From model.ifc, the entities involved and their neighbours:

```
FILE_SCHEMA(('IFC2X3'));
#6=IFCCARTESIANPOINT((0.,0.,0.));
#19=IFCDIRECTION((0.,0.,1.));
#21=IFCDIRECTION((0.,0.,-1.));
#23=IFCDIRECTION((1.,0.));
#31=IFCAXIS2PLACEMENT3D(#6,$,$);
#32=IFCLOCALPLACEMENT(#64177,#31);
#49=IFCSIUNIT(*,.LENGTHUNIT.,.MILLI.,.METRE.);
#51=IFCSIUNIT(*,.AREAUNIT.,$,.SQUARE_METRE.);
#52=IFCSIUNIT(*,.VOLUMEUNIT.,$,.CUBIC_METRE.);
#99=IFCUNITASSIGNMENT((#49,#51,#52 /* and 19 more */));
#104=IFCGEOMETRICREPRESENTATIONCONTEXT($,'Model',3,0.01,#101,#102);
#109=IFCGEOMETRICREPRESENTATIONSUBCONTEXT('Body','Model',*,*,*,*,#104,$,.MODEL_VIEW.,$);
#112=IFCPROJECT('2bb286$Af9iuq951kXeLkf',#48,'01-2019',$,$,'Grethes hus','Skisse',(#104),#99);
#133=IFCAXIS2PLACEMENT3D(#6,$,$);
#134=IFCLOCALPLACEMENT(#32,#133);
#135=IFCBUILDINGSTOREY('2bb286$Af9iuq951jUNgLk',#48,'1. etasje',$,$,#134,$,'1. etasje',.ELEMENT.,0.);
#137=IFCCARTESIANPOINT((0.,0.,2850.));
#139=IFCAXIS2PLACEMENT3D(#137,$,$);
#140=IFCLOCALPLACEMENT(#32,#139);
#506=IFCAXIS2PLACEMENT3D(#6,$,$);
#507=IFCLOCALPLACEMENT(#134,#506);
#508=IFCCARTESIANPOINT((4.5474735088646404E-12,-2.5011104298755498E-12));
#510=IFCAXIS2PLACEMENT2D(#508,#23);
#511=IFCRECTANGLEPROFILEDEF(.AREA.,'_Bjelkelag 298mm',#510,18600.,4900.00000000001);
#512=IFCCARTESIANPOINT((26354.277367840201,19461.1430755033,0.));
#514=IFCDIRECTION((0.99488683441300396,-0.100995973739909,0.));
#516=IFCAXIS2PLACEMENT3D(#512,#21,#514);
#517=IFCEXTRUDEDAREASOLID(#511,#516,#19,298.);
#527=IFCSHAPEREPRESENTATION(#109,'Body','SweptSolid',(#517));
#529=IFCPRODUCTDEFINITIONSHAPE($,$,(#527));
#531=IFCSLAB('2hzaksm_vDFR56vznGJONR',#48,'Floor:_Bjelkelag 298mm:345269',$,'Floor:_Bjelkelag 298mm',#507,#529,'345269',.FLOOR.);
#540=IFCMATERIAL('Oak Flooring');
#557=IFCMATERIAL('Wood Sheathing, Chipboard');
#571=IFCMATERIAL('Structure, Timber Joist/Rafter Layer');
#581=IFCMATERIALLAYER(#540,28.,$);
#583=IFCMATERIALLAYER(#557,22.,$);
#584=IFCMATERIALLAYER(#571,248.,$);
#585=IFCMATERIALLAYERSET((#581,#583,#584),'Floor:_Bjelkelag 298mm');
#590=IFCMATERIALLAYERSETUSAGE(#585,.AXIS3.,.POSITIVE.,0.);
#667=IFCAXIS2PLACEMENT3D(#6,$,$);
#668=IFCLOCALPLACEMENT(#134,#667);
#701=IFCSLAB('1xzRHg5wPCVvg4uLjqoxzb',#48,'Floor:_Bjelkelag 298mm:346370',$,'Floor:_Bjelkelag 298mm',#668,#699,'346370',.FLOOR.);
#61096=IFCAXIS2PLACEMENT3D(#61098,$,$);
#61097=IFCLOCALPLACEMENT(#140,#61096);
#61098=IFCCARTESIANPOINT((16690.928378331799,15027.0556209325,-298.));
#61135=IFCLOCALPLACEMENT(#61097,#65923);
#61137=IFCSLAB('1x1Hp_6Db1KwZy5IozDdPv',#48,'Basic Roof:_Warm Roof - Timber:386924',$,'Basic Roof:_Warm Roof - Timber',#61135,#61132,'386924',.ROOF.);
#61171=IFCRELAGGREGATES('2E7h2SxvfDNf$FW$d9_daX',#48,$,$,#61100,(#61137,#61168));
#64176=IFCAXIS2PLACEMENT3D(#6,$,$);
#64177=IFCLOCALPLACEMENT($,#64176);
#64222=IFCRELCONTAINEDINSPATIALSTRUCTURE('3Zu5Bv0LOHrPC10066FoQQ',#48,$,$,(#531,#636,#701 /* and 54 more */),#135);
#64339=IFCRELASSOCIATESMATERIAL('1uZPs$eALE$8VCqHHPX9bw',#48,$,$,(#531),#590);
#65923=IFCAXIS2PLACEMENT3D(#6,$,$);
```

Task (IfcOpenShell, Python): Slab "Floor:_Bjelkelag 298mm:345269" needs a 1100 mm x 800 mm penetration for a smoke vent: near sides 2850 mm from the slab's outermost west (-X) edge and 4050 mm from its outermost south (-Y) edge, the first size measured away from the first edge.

```python
import numpy as np
import ifcopenshell
import ifcopenshell.api.feature
import ifcopenshell.api.geometry
import ifcopenshell.api.root
import ifcopenshell.geom
import ifcopenshell.util.placement
import ifcopenshell.util.representation
import ifcopenshell.util.shape
import ifcopenshell.util.unit

model = ifcopenshell.open("model.ifc")
unit_scale = ifcopenshell.util.unit.calculate_unit_scale(model)
settings = ifcopenshell.geom.settings()


def volume(element):
    """Net volume in cubic metres, openings subtracted."""
    shape = ifcopenshell.geom.create_shape(settings, element)
    return ifcopenshell.util.shape.get_volume(shape.geometry)


slab = model.by_guid("2hzaksm_vDFR56vznGJONR")
before = volume(slab)

# Extent in the slab's own axes, in metres. The edges named are its -X and -Y sides.
slab_shape = ifcopenshell.geom.create_shape(settings, slab)
vertices = ifcopenshell.util.shape.get_vertices(slab_shape.geometry)
x_min, y_min, bottom = vertices.min(axis=0)
top = vertices[:, 2].max()

opening = ifcopenshell.api.root.create_entity(model, ifc_class="IfcOpeningElement", name="Smoke vent opening")
context = ifcopenshell.util.representation.get_context(model, "Model", "Body", "MODEL_VIEW")
width, depth = 1.1, 0.8
outline = [(0.0, 0.0), (width, 0.0), (width, depth), (0.0, depth), (0.0, 0.0)]
# Overshoot both faces by 50 mm so the cut is clean.
shape = ifcopenshell.api.geometry.add_slab_representation(
    model, context=context, depth=top - bottom + 0.1, polyline=outline
)
ifcopenshell.api.geometry.assign_representation(model, product=opening, representation=shape)

matrix = ifcopenshell.util.placement.get_local_placement(slab.ObjectPlacement)
matrix[:, 3] = matrix @ np.append(np.array([x_min + 2.85, y_min + 4.05, bottom - 0.05]) / unit_scale, 1.0)
ifcopenshell.api.geometry.edit_object_placement(model, product=opening, matrix=matrix, is_si=False)
ifcopenshell.api.feature.add_feature(model, feature=opening, element=slab)

after = volume(slab)

print(f"slab volume {before:.3f} -> {after:.3f} m3")

model.write("model_edited.ifc")
```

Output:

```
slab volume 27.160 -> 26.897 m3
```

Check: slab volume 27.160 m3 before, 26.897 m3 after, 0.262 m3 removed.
